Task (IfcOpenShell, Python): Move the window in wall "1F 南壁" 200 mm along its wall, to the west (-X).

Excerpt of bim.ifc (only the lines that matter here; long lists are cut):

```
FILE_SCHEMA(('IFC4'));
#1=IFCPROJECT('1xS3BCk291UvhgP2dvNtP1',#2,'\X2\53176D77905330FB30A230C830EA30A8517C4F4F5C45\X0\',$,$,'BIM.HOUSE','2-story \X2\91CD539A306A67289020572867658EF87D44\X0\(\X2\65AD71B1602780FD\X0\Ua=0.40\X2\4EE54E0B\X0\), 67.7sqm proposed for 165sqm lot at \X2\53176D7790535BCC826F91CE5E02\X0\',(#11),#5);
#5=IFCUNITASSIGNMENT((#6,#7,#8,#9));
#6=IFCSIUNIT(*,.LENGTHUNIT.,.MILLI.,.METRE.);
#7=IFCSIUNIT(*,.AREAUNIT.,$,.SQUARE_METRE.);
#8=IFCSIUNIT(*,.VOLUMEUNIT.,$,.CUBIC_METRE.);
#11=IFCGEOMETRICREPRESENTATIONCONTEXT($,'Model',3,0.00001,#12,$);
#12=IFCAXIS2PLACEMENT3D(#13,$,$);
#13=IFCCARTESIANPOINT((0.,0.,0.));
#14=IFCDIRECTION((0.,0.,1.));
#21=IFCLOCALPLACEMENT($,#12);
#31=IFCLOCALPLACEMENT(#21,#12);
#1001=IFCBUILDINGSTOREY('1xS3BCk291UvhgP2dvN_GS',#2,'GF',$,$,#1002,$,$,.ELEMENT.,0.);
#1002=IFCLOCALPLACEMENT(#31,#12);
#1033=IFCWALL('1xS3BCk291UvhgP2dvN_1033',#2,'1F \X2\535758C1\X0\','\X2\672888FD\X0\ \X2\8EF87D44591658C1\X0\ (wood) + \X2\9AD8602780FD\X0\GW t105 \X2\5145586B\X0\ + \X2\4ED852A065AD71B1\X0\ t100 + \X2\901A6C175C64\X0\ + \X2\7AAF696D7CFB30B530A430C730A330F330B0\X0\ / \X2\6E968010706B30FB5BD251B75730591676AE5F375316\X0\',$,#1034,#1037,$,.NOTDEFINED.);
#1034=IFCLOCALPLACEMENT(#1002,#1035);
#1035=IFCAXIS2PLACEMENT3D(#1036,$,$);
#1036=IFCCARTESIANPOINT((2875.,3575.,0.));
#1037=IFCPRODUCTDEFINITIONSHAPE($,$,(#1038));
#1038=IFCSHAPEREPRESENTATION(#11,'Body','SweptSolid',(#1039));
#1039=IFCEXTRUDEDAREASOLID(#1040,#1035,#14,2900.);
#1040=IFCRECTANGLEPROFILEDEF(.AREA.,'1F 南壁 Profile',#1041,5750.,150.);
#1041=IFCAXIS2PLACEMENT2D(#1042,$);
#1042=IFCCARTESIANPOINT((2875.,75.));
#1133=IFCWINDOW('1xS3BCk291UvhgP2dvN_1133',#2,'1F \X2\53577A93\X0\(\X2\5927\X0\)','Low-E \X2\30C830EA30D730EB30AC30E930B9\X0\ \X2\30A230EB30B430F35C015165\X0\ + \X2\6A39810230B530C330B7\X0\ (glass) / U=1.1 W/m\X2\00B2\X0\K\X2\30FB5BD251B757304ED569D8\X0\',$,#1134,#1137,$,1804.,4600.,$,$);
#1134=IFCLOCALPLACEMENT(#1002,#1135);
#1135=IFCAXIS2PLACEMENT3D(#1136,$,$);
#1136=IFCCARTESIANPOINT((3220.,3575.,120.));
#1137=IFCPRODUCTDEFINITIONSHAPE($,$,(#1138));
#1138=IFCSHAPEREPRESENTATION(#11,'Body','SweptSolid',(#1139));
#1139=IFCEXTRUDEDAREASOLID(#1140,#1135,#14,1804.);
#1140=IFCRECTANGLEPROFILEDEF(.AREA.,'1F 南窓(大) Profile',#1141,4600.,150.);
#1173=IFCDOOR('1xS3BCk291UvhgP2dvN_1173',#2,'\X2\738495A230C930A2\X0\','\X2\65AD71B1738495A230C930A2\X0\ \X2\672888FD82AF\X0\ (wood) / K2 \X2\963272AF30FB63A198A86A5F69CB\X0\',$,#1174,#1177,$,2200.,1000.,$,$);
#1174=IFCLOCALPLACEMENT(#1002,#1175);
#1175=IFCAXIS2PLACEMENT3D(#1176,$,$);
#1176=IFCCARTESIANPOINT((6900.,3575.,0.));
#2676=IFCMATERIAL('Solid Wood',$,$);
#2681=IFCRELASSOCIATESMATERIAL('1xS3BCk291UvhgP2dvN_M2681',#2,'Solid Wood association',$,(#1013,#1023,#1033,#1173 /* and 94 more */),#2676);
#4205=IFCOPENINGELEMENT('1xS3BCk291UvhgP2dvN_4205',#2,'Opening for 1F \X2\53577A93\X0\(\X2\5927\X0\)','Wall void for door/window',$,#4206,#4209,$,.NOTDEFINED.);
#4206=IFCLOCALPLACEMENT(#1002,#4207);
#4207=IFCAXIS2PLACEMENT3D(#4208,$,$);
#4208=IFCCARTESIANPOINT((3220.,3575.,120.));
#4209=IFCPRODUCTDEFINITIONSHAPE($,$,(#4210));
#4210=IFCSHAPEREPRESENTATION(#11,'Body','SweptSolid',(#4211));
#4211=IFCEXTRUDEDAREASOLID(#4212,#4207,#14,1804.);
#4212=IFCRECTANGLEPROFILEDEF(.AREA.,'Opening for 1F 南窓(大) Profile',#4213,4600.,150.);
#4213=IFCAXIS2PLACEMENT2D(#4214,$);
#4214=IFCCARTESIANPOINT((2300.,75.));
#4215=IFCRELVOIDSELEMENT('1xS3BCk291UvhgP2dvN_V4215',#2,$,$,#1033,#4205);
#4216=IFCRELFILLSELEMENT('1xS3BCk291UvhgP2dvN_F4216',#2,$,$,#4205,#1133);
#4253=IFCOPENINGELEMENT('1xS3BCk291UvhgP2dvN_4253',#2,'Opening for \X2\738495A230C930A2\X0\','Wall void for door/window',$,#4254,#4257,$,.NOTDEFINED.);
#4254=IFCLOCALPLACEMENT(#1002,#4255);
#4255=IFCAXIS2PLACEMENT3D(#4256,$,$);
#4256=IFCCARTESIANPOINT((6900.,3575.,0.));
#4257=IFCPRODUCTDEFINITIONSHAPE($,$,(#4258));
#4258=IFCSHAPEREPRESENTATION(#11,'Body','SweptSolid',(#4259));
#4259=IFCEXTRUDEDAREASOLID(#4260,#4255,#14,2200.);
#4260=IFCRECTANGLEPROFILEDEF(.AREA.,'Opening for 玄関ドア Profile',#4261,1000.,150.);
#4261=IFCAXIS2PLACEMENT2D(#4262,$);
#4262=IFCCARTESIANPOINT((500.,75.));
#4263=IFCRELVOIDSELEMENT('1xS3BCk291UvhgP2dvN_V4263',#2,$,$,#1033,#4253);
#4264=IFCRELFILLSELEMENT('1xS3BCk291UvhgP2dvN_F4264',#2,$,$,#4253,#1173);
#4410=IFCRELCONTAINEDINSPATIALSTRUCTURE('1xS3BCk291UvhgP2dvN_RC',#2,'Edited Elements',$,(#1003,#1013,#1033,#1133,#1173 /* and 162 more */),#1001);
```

```python
import ifcopenshell
import ifcopenshell.api.geometry
import ifcopenshell.util.placement
import ifcopenshell.util.unit

model = ifcopenshell.open("bim.ifc")
unit_scale = ifcopenshell.util.unit.calculate_unit_scale(model)

window = model.by_guid("1xS3BCk291UvhgP2dvN_1133")
opening = window.FillsVoids[0].RelatingOpeningElement
wall = opening.VoidsElements[0].RelatingBuildingElement

wall_matrix = ifcopenshell.util.placement.get_local_placement(wall.ObjectPlacement)
shift = wall_matrix[:3, 0] * -0.2 / unit_scale
before = ifcopenshell.util.placement.get_local_placement(window.ObjectPlacement)[:3, 3].copy()

# The window is not placed relative to its opening, so move both.
for product in (opening, window):
    matrix = ifcopenshell.util.placement.get_local_placement(product.ObjectPlacement)
    matrix[:3, 3] += shift
    ifcopenshell.api.geometry.edit_object_placement(model, product=product, matrix=matrix, is_si=False)

after = ifcopenshell.util.placement.get_local_placement(window.ObjectPlacement)[:3, 3]
print("window moved by", (after - before).round(3) + 0.0)

model.write("bim_updated.ifc")
```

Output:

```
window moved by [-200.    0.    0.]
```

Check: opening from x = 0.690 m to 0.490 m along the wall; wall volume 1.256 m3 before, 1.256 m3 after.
